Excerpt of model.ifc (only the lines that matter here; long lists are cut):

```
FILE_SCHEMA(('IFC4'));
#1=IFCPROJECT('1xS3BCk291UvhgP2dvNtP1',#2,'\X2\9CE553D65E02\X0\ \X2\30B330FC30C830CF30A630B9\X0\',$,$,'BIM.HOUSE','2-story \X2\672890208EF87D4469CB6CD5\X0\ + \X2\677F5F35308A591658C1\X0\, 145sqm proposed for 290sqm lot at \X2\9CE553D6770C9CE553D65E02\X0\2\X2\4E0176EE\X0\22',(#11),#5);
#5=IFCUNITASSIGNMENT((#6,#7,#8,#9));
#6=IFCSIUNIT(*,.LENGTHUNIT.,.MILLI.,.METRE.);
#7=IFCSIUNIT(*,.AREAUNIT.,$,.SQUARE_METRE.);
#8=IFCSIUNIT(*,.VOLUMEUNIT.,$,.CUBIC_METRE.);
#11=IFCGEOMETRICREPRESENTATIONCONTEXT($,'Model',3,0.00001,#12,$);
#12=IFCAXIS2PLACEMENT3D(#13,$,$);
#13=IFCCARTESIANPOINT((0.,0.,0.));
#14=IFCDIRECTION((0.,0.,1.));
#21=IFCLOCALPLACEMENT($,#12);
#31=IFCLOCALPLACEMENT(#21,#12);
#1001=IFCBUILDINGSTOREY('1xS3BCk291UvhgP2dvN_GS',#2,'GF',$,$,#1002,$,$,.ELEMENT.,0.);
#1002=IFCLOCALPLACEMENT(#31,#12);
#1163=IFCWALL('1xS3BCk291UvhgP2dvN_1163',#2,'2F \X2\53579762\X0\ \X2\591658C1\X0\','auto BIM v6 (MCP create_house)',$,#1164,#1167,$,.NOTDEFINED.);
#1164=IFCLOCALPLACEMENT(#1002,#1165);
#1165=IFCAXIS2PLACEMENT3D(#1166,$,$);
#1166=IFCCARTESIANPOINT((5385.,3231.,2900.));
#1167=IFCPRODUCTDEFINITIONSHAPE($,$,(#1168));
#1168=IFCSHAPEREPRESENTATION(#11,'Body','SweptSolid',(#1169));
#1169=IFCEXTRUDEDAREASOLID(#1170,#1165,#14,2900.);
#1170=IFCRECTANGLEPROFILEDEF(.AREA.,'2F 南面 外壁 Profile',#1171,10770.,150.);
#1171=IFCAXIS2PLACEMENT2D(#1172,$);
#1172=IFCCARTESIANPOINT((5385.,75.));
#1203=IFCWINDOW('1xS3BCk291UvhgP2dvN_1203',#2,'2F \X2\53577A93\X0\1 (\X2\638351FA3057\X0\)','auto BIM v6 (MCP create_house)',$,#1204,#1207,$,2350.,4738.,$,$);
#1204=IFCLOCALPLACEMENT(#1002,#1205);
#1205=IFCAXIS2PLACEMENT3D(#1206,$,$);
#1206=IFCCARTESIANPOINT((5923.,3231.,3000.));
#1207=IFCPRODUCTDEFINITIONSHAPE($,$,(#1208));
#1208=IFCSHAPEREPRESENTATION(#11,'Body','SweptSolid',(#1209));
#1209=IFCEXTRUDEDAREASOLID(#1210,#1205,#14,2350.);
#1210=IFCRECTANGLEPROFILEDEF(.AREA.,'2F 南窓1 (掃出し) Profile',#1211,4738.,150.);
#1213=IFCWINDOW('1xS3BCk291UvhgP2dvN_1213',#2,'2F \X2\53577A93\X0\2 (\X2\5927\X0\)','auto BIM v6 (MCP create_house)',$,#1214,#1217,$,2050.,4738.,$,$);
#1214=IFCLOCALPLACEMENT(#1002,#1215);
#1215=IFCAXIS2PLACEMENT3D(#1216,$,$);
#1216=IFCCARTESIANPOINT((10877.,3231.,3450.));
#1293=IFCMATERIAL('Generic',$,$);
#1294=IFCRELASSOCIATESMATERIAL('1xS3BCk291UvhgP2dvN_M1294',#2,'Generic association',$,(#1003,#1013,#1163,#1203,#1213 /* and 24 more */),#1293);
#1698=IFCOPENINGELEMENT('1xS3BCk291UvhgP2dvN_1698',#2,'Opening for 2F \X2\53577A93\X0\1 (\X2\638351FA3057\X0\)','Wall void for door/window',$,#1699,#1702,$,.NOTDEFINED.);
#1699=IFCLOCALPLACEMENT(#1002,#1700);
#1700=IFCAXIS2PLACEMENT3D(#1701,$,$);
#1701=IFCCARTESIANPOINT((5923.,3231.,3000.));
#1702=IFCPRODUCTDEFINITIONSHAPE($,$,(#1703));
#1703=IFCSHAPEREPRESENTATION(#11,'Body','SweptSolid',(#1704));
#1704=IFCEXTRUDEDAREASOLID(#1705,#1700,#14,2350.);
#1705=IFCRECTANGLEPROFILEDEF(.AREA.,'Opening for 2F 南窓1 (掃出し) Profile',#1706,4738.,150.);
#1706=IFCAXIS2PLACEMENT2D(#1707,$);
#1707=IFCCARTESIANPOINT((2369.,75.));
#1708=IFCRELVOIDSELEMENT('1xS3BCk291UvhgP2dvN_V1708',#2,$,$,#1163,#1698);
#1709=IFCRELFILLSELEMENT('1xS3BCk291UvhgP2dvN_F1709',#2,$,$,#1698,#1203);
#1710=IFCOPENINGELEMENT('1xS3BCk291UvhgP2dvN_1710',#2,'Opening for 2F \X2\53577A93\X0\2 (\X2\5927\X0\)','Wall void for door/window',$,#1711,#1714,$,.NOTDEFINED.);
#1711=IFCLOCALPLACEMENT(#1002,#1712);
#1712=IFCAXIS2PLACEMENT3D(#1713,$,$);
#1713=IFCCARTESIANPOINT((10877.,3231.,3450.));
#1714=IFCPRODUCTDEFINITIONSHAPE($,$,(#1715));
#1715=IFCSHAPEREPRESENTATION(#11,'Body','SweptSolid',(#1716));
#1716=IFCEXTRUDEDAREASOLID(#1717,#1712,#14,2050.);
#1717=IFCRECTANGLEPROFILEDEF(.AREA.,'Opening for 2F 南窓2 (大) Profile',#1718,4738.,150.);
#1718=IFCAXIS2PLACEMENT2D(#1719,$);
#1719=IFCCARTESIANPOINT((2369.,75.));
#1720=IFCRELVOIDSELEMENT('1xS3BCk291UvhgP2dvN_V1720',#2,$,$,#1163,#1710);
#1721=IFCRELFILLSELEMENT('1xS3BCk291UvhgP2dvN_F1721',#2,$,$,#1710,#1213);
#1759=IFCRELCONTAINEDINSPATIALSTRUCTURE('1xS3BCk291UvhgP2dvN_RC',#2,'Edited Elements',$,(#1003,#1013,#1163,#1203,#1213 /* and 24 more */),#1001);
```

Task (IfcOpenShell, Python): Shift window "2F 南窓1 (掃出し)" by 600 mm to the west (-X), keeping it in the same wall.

```python
import ifcopenshell
import ifcopenshell.api.geometry
import ifcopenshell.util.placement
import ifcopenshell.util.unit

model = ifcopenshell.open("model.ifc")
unit_scale = ifcopenshell.util.unit.calculate_unit_scale(model)

window = model.by_guid("1xS3BCk291UvhgP2dvN_1203")
opening = window.FillsVoids[0].RelatingOpeningElement
wall = opening.VoidsElements[0].RelatingBuildingElement

wall_matrix = ifcopenshell.util.placement.get_local_placement(wall.ObjectPlacement)
shift = wall_matrix[:3, 0] * -0.6 / unit_scale
before = ifcopenshell.util.placement.get_local_placement(window.ObjectPlacement)[:3, 3].copy()

# The window is not placed relative to its opening, so move both.
for product in (opening, window):
    matrix = ifcopenshell.util.placement.get_local_placement(product.ObjectPlacement)
    matrix[:3, 3] += shift
    ifcopenshell.api.geometry.edit_object_placement(model, product=product, matrix=matrix, is_si=False)

after = ifcopenshell.util.placement.get_local_placement(window.ObjectPlacement)[:3, 3]
print("window moved by", (after - before).round(3) + 0.0)

model.write("model_edited.ifc")
```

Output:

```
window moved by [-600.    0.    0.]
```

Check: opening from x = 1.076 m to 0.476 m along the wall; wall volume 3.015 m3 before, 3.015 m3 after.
